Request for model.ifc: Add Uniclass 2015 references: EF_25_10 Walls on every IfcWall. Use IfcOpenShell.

First a look at what the model holds.

```python
import ifcopenshell

model = ifcopenshell.open("model.ifc")
print(model.schema)
print("classifications:", [c.Name for c in model.by_type("IfcClassification")])
for ifc_class in ("IfcDoor", "IfcRoof", "IfcStair", "IfcWall", "IfcWindow"):
    print(ifc_class, len(model.by_type(ifc_class)))
```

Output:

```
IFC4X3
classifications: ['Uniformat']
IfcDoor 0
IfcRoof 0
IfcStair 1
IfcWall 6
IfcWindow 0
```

```python
import ifcopenshell
import ifcopenshell.api.classification

model = ifcopenshell.open("model.ifc")

system = ifcopenshell.api.classification.add_classification(model, classification="Uniclass 2015")

codes = {
    "IfcWall": ("EF_25_10", "Walls"),
}
for ifc_class, (code, name) in codes.items():
    products = model.by_type(ifc_class)
    ifcopenshell.api.classification.add_reference(
        model, products=products, classification=system, identification=code, name=name
    )
    print(code, len(products))

model.write("model_edited.ifc")
```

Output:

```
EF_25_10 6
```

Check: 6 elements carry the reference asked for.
